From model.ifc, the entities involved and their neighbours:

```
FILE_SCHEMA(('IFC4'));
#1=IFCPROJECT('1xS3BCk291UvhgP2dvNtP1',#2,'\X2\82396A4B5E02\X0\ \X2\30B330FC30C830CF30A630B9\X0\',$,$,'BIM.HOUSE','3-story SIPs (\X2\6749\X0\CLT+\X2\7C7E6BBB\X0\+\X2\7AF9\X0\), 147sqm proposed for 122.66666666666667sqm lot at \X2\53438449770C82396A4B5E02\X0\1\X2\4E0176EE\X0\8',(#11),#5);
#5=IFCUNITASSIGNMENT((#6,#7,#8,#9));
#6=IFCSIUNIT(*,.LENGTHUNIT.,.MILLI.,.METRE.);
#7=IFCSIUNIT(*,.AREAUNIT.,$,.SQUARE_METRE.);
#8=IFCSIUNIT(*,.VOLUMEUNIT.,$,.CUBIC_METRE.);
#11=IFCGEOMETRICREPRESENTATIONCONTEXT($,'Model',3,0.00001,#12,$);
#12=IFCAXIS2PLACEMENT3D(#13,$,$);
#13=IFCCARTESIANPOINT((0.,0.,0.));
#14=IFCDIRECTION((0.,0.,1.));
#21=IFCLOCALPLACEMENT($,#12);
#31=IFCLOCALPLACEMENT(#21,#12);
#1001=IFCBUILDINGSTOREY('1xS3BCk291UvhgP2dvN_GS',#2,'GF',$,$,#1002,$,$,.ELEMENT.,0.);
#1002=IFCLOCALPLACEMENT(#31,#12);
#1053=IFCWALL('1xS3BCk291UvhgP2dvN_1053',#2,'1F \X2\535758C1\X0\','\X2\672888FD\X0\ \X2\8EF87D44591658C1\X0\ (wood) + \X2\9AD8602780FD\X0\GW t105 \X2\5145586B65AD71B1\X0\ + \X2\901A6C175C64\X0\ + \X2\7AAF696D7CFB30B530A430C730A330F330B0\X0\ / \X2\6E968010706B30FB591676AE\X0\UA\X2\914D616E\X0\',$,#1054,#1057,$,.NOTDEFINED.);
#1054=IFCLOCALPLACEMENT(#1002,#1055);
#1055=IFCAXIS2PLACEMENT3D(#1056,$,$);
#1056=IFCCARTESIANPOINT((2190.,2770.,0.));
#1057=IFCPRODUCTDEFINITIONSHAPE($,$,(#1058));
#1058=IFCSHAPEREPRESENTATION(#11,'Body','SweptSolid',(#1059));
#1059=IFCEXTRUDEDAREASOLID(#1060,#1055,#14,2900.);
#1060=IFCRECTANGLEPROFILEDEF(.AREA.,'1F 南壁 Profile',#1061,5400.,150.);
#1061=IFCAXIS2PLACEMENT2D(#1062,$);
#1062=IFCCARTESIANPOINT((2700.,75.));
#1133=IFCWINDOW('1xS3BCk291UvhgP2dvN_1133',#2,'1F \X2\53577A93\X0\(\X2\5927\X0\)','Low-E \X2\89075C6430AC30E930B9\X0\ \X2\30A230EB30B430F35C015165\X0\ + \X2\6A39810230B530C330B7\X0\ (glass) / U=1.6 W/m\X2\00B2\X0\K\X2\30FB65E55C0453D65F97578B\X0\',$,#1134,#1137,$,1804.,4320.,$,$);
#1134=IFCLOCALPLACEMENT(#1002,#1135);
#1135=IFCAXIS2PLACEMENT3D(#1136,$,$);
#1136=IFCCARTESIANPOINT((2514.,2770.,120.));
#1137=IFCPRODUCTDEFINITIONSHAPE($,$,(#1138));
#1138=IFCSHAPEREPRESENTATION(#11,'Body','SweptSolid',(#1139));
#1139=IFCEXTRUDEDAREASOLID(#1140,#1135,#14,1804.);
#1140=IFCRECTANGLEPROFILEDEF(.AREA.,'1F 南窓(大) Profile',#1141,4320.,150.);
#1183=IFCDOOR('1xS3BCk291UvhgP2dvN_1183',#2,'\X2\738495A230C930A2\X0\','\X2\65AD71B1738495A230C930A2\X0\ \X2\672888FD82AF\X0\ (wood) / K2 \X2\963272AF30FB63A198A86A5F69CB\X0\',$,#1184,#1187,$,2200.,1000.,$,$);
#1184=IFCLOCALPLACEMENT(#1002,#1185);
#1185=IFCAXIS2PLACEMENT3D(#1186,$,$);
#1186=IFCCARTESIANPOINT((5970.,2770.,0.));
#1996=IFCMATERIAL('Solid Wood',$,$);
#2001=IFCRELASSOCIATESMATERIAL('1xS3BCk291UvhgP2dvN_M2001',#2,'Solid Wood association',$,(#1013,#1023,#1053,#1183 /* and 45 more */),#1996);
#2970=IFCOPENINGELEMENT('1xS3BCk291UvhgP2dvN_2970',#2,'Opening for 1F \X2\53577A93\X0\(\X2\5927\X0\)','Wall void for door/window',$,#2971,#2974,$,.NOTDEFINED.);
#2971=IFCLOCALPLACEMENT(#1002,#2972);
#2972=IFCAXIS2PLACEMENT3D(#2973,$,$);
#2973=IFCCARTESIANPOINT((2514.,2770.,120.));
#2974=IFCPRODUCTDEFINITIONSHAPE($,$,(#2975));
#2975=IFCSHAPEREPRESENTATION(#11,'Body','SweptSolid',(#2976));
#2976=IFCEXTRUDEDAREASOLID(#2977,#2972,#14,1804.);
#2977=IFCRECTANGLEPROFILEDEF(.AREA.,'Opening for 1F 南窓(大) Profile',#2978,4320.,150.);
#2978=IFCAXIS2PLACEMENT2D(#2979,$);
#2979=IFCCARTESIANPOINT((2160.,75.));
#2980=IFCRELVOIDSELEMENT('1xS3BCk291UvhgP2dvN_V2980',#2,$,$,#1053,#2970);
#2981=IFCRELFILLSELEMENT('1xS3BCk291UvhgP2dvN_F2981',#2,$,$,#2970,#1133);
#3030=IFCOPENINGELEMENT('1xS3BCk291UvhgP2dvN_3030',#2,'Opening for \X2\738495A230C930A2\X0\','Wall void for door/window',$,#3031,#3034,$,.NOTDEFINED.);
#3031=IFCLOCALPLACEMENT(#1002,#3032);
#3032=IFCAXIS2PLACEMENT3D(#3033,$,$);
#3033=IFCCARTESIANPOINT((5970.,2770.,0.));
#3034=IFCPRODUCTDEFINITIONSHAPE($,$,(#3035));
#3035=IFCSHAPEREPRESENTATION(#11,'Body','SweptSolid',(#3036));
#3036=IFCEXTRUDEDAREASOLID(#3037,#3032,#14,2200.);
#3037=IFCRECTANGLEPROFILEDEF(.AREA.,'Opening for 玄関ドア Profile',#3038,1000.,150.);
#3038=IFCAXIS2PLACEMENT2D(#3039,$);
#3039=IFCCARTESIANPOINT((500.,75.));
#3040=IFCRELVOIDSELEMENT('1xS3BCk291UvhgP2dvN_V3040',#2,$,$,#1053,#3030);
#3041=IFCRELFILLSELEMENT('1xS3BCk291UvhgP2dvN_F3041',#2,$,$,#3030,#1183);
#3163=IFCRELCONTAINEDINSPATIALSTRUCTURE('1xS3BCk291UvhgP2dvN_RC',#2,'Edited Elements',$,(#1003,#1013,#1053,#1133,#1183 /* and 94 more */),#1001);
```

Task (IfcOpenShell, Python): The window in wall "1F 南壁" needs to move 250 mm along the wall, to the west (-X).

```python
import ifcopenshell
import ifcopenshell.api.geometry
import ifcopenshell.util.placement

model = ifcopenshell.open("model.ifc")

window = model.by_guid("1xS3BCk291UvhgP2dvN_1133")
opening = window.FillsVoids[0].RelatingOpeningElement
wall = opening.VoidsElements[0].RelatingBuildingElement

wall_matrix = ifcopenshell.util.placement.get_local_placement(wall.ObjectPlacement)
shift = wall_matrix[:3, 0] * -250.0
before = ifcopenshell.util.placement.get_local_placement(window.ObjectPlacement)[:3, 3].copy()

# The window is not placed relative to its opening, so move both.
for product in (opening, window):
    matrix = ifcopenshell.util.placement.get_local_placement(product.ObjectPlacement)
    matrix[:3, 3] += shift
    ifcopenshell.api.geometry.edit_object_placement(model, product=product, matrix=matrix, is_si=False)

after = ifcopenshell.util.placement.get_local_placement(window.ObjectPlacement)[:3, 3]
print("window moved by", (after - before).round(3) + 0.0)

model.write("model_v2.ifc")
```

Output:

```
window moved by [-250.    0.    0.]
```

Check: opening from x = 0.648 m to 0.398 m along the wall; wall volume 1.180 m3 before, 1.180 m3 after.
